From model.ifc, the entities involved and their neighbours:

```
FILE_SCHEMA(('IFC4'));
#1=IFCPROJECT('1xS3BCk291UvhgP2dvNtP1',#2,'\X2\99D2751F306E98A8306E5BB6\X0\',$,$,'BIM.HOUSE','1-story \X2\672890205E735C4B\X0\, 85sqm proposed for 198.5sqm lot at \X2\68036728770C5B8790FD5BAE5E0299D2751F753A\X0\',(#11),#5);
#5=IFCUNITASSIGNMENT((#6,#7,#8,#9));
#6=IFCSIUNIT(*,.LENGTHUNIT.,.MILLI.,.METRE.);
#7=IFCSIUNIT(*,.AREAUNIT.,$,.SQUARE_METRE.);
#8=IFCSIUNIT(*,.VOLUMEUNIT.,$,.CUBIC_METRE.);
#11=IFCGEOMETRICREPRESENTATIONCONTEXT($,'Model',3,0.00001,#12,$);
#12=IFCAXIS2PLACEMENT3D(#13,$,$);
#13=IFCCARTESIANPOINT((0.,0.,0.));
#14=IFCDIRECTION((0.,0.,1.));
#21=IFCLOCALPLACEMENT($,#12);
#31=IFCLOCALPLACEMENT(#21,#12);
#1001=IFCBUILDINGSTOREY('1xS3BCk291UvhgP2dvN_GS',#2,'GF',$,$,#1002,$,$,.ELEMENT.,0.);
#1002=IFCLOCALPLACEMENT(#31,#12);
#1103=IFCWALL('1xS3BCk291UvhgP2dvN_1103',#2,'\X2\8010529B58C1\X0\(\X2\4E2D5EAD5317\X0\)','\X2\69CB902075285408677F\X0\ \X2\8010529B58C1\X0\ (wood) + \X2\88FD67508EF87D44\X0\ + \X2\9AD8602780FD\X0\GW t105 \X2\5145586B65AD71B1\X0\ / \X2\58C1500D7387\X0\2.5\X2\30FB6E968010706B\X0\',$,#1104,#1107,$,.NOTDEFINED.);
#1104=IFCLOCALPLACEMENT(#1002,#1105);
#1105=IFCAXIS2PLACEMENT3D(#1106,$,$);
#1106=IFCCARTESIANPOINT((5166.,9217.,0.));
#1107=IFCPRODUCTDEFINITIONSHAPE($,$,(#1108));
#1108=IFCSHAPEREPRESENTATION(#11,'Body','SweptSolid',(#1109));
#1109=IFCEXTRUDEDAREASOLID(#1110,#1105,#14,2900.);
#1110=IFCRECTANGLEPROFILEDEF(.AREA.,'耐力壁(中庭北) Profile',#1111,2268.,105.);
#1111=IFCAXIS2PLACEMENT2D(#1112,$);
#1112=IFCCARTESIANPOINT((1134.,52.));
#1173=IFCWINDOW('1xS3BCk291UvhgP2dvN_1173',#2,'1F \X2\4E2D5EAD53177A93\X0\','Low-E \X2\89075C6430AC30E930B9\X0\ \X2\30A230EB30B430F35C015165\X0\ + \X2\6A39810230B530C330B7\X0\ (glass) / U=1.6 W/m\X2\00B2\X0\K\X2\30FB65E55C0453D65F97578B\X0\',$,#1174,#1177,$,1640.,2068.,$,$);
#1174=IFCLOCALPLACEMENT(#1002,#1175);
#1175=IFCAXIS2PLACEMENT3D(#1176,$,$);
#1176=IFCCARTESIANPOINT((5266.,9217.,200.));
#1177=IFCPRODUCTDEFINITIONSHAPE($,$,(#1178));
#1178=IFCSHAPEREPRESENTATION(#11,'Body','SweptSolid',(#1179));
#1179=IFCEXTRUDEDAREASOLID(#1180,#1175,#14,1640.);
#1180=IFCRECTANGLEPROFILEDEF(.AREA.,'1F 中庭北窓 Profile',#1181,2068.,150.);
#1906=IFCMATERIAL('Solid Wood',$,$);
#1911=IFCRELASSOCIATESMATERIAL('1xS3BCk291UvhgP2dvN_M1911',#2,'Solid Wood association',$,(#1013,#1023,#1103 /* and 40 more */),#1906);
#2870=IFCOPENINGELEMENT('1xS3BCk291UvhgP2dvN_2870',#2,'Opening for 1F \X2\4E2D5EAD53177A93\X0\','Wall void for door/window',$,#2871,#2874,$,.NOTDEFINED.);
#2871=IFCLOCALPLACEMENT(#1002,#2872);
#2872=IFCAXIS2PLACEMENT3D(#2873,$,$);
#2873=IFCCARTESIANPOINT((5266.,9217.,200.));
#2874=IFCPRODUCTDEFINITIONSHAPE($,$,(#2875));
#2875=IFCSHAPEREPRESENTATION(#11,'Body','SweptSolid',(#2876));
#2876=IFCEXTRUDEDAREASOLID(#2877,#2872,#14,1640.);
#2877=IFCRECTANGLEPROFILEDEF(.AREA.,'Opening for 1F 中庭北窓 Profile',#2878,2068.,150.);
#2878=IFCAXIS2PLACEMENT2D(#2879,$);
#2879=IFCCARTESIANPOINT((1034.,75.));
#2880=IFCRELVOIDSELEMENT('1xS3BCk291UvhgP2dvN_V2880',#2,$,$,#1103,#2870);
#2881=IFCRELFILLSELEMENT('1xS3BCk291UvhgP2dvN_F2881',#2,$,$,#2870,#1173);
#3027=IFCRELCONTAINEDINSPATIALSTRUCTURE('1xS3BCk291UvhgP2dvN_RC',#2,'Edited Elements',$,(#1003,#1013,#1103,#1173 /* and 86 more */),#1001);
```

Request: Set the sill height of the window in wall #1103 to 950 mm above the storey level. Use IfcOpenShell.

```python
import numpy as np
import ifcopenshell
import ifcopenshell.api.geometry
import ifcopenshell.geom
import ifcopenshell.util.element
import ifcopenshell.util.placement
import ifcopenshell.util.shape
import ifcopenshell.util.unit

model = ifcopenshell.open("model.ifc")
unit_scale = ifcopenshell.util.unit.calculate_unit_scale(model)

window = model.by_id(1173)
opening = window.FillsVoids[0].RelatingOpeningElement
storey = ifcopenshell.util.element.get_container(window, ifc_class="IfcBuildingStorey")
level = ifcopenshell.util.placement.get_local_placement(storey.ObjectPlacement)[2, 3]

# The opening's origin need not be at the sill, so measure its lowest point.
shape = ifcopenshell.geom.create_shape(ifcopenshell.geom.settings(), opening)
bottom = ifcopenshell.util.shape.get_shape_bottom_elevation(shape, shape.geometry) / unit_scale
dz = level + 0.95 / unit_scale - bottom

shift = np.array([0.0, 0.0, dz])
# The window is not placed relative to its opening, so move both.
for product in (opening, window):
    matrix = ifcopenshell.util.placement.get_local_placement(product.ObjectPlacement)
    matrix[:3, 3] += shift
    ifcopenshell.api.geometry.edit_object_placement(model, product=product, matrix=matrix, is_si=False)

print(f"moved by {dz * unit_scale:+.3f} m")

model.write("model-out.ifc")
```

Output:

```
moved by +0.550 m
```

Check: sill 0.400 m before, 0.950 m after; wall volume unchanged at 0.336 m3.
